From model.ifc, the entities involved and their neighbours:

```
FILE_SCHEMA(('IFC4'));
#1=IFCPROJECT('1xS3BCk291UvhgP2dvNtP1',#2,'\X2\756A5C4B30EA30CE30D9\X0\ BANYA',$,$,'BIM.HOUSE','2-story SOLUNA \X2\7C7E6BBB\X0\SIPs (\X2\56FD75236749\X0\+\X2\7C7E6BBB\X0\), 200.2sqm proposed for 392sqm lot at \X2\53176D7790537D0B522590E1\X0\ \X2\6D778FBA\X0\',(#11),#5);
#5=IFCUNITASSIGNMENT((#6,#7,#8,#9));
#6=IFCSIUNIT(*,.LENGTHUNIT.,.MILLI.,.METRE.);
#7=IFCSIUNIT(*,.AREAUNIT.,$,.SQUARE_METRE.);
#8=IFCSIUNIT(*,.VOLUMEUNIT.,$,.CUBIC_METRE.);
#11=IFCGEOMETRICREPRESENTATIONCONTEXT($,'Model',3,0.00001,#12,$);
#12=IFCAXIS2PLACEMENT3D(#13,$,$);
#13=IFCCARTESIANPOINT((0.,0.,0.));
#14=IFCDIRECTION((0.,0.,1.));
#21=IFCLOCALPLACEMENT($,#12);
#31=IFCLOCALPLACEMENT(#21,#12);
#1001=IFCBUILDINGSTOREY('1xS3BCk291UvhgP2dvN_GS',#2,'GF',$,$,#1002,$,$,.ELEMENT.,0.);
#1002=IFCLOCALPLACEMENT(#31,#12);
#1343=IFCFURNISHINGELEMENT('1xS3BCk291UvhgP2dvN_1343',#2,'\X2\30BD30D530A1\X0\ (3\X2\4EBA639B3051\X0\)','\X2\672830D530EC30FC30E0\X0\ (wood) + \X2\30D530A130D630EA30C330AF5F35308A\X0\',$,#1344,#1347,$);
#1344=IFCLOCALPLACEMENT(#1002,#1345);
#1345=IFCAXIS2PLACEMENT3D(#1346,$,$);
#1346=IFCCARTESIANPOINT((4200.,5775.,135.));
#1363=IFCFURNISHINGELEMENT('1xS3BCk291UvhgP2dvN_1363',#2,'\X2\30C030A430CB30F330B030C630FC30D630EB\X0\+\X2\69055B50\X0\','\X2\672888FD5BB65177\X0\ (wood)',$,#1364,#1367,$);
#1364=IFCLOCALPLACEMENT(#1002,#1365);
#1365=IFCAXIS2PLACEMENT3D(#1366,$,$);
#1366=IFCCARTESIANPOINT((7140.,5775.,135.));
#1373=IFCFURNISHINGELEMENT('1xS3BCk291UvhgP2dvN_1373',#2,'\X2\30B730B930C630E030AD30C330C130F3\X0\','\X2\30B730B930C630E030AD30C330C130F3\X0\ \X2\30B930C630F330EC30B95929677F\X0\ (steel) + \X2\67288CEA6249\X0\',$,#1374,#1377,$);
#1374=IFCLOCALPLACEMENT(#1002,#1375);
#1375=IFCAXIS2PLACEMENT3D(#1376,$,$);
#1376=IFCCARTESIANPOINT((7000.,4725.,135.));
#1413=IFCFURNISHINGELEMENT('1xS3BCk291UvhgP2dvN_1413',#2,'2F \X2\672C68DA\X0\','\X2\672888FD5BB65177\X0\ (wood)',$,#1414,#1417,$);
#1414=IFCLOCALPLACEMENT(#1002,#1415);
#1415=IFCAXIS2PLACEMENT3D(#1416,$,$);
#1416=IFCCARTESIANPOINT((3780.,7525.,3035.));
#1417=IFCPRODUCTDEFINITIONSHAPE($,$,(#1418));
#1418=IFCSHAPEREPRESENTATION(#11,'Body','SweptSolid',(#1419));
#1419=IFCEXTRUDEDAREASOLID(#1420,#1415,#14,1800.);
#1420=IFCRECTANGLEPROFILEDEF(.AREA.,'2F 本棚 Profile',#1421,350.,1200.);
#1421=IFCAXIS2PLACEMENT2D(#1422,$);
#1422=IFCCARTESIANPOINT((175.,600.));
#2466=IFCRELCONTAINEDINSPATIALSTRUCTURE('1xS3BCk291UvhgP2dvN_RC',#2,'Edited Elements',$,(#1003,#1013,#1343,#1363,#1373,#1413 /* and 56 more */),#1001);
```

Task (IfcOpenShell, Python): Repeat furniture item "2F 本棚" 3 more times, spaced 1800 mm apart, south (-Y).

```python
import numpy as np
import ifcopenshell
import ifcopenshell.api.geometry
import ifcopenshell.api.root
import ifcopenshell.util.element
import ifcopenshell.util.placement
import ifcopenshell.util.unit

model = ifcopenshell.open("model.ifc")
unit_scale = ifcopenshell.util.unit.calculate_unit_scale(model)


def reuse_history(source, copy):
    """copy_class also copies each property set's owner history, people and application; keep the originals."""
    for rel in copy.IsDefinedBy:
        if rel.is_a("IfcRelDefinesByProperties") and (history := rel.RelatingPropertyDefinition.OwnerHistory):
            rel.RelatingPropertyDefinition.OwnerHistory = source.OwnerHistory
            ifcopenshell.util.element.remove_deep2(model, history)


source = model.by_guid("1xS3BCk291UvhgP2dvN_1413")
base = ifcopenshell.util.placement.get_local_placement(source.ObjectPlacement)
step = np.array([0.0, -1.0, 0.0]) * 1.8 / unit_scale

for i in range(1, 4):
    copy = ifcopenshell.api.root.copy_class(model, product=source)
    copy.Representation = ifcopenshell.util.element.copy_deep(
        model, source.Representation, exclude=["IfcGeometricRepresentationContext", "IfcRepresentationMap"]
    )
    reuse_history(source, copy)
    matrix = base.copy()
    matrix[:3, 3] += i * step
    print("added at", matrix[:3, 3].round(3) + 0.0)
    ifcopenshell.api.geometry.edit_object_placement(model, product=copy, matrix=matrix, is_si=False)

model.write("model_edited.ifc")
```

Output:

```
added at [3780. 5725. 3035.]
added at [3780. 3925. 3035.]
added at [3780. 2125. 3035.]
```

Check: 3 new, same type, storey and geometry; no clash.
